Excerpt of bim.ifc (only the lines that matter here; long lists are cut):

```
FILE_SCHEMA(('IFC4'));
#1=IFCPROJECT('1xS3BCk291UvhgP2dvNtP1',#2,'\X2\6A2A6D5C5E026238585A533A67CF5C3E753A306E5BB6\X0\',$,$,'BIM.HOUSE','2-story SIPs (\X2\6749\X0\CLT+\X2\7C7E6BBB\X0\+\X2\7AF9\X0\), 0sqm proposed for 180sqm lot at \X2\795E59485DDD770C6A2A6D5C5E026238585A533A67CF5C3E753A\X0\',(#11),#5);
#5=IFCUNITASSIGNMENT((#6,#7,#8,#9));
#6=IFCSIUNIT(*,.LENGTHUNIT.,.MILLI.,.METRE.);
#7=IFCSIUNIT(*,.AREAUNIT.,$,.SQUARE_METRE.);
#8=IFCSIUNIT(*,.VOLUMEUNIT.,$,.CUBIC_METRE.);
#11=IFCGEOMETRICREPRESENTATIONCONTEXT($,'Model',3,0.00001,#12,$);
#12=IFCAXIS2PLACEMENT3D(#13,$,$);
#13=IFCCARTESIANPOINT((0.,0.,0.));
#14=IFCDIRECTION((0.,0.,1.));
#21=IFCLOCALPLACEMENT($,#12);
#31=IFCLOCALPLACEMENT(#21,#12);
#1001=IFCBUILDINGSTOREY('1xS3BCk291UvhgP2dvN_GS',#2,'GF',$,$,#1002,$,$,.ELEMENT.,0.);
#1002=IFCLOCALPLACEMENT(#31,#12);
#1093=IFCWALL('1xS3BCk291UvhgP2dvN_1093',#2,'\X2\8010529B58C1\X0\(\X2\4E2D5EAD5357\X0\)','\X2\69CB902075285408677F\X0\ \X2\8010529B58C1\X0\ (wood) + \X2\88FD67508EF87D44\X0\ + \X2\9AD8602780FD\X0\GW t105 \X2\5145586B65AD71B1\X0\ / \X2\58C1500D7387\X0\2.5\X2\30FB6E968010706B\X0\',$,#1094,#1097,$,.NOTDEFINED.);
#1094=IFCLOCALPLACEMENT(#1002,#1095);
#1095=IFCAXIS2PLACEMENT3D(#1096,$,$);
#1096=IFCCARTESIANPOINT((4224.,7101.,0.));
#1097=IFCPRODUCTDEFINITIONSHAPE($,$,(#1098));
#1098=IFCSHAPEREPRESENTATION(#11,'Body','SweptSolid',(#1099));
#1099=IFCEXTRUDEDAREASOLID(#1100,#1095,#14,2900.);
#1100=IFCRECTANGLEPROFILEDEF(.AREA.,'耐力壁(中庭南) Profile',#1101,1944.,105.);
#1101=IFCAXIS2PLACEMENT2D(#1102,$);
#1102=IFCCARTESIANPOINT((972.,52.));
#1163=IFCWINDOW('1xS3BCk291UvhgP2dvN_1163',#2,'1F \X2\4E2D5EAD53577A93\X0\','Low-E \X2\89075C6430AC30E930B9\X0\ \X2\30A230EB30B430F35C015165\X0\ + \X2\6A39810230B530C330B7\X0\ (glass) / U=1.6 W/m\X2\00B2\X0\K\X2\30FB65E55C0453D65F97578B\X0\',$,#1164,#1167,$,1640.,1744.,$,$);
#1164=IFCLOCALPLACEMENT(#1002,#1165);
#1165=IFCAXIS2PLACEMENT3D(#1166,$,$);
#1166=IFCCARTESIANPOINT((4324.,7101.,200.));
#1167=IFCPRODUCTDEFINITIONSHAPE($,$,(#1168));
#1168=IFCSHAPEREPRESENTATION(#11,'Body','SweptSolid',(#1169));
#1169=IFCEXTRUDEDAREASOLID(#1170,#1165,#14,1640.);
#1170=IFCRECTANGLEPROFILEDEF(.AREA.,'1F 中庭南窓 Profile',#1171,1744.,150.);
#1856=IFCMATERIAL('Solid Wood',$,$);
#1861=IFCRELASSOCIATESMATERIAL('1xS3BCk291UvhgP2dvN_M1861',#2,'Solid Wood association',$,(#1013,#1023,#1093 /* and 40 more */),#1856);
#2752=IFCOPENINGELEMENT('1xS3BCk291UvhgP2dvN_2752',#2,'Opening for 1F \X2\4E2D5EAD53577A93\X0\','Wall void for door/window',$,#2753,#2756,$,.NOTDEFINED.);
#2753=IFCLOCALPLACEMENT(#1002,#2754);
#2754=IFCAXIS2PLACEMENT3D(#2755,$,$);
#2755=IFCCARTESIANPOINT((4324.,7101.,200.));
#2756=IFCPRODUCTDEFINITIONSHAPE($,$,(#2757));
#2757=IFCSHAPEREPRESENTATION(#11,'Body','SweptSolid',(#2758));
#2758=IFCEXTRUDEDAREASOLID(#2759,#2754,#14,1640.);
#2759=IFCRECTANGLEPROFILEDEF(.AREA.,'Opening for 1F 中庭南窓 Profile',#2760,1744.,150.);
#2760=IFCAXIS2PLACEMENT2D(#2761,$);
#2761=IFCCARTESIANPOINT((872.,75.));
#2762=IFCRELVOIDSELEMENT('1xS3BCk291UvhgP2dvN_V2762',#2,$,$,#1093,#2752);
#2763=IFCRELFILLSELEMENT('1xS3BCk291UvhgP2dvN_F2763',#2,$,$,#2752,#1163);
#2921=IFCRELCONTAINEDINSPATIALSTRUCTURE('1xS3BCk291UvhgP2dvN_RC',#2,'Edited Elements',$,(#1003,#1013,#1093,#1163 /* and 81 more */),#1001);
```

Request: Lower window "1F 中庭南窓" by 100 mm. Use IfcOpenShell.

```python
import numpy as np
import ifcopenshell
import ifcopenshell.api.geometry
import ifcopenshell.util.placement
import ifcopenshell.util.unit

model = ifcopenshell.open("bim.ifc")
unit_scale = ifcopenshell.util.unit.calculate_unit_scale(model)

window = model.by_guid("1xS3BCk291UvhgP2dvN_1163")
opening = window.FillsVoids[0].RelatingOpeningElement
dz = -0.1 / unit_scale

shift = np.array([0.0, 0.0, dz])
# The window is not placed relative to its opening, so move both.
for product in (opening, window):
    matrix = ifcopenshell.util.placement.get_local_placement(product.ObjectPlacement)
    matrix[:3, 3] += shift
    ifcopenshell.api.geometry.edit_object_placement(model, product=product, matrix=matrix, is_si=False)

print(f"moved by {dz * unit_scale:+.3f} m")

model.write("bim_updated.ifc")
```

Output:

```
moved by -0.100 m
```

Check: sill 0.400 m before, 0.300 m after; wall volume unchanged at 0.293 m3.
